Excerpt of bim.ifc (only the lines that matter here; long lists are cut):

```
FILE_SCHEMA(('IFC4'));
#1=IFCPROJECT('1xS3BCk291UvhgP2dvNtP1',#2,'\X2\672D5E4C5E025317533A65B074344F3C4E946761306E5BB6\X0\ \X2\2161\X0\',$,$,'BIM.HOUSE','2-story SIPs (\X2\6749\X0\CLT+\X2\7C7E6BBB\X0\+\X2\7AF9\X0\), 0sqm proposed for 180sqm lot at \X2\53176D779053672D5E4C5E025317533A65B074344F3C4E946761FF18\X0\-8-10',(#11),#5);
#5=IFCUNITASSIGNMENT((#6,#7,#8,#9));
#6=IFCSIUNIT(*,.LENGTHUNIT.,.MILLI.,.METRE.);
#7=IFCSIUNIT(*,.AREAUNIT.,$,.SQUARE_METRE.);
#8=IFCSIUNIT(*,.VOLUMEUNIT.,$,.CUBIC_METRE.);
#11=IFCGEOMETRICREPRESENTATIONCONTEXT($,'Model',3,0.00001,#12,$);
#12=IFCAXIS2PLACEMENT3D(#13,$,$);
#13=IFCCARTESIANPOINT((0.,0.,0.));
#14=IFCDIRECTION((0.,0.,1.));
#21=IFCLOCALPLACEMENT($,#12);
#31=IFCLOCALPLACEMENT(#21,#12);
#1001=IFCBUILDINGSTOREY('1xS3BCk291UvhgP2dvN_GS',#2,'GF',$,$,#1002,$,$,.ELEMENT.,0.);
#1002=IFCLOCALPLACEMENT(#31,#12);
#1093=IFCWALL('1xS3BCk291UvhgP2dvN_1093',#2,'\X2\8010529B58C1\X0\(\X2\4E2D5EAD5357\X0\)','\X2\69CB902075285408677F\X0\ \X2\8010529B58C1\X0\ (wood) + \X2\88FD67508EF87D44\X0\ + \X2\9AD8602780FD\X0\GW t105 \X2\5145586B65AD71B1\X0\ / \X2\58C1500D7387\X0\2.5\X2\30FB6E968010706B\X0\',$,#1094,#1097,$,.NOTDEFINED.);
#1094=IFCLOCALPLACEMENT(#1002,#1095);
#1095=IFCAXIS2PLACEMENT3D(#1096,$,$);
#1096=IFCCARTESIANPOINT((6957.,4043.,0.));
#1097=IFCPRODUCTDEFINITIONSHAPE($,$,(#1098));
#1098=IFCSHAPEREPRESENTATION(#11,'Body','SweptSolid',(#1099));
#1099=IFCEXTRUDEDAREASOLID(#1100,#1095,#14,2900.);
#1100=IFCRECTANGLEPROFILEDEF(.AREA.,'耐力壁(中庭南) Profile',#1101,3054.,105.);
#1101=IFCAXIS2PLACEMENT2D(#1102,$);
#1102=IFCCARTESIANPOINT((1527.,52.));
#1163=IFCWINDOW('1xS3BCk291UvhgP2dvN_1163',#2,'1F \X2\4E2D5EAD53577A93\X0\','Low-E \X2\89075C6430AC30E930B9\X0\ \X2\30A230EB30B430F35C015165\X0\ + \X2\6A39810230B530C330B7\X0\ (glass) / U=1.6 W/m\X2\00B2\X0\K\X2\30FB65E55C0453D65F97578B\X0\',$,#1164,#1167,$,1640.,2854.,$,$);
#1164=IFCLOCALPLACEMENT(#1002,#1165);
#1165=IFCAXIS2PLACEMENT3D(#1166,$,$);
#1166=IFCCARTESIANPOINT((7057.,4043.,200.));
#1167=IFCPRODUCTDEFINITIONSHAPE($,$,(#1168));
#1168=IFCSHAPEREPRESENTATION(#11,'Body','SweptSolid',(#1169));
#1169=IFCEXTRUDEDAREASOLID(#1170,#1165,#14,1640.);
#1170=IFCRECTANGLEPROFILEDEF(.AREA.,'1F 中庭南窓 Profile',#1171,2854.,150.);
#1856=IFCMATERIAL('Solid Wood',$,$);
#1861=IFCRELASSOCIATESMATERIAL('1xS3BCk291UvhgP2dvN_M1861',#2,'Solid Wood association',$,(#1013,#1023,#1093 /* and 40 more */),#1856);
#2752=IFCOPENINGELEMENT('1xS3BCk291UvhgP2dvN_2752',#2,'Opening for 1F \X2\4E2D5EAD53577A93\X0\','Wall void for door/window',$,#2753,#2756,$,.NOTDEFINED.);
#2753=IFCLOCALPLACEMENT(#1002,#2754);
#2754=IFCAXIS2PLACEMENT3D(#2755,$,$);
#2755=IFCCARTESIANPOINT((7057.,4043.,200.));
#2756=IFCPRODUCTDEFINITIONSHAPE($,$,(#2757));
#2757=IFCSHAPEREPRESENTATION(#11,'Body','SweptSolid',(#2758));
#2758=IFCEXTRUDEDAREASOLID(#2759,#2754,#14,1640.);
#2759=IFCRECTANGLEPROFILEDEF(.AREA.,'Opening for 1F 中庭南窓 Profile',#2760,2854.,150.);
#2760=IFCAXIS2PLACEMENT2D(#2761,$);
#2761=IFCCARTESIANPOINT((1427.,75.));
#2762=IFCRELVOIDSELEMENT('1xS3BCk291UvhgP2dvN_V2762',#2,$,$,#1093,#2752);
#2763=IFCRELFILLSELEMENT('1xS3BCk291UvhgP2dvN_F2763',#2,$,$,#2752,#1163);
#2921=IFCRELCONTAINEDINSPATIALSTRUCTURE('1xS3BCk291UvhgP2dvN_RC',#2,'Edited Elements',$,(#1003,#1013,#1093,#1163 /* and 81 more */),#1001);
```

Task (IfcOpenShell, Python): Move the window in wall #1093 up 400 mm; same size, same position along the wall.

```python
import numpy as np
import ifcopenshell
import ifcopenshell.api.geometry
import ifcopenshell.util.placement
import ifcopenshell.util.unit

model = ifcopenshell.open("bim.ifc")
unit_scale = ifcopenshell.util.unit.calculate_unit_scale(model)

window = model.by_guid("1xS3BCk291UvhgP2dvN_1163")
opening = window.FillsVoids[0].RelatingOpeningElement
dz = 400.0

shift = np.array([0.0, 0.0, dz])
# The window is not placed relative to its opening, so move both.
for product in (opening, window):
    matrix = ifcopenshell.util.placement.get_local_placement(product.ObjectPlacement)
    matrix[:3, 3] += shift
    ifcopenshell.api.geometry.edit_object_placement(model, product=product, matrix=matrix, is_si=False)

print(f"moved by {dz * unit_scale:+.3f} m")

model.write("bim_v2.ifc")
```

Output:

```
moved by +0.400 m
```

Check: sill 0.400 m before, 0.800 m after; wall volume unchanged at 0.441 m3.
